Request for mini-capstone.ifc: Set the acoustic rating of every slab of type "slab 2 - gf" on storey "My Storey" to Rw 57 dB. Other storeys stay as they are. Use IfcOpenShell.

First a look at what the model holds.

```python
import ifcopenshell
import ifcopenshell.util.element

model = ifcopenshell.open("mini-capstone.ifc")
print(model.schema)
storey = next(s for s in model.by_type("IfcBuildingStorey") if s.Name == "My Storey")
slabs = [e for e in ifcopenshell.util.element.get_decomposition(storey) if e.is_a("IfcSlab")]
seen = {}
for e in slabs:
    element_type = ifcopenshell.util.element.get_type(e)
    key = (element_type.Name if element_type != e and element_type else None, ifcopenshell.util.element.get_pset(e, "Pset_SlabCommon", "AcousticRating"))
    seen[key] = seen.get(key, 0) + 1
for (name, value), count in sorted(seen.items(), key=str):
    print(count, "x", name, "|", value)
```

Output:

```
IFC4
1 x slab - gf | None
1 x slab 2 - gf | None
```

```python
import ifcopenshell
import ifcopenshell.api.pset
import ifcopenshell.util.element

model = ifcopenshell.open("mini-capstone.ifc")

storey = next(s for s in model.by_type("IfcBuildingStorey") if s.Name == "My Storey")
slabs = [e for e in ifcopenshell.util.element.get_decomposition(storey) if e.is_a("IfcSlab")]

count = 0
for e in slabs:
    element_type = ifcopenshell.util.element.get_type(e)
    if element_type in (None, e) or element_type.Name != "slab 2 - gf":
        continue
    # add_pset returns the element's existing set when there is one.
    pset = ifcopenshell.api.pset.add_pset(model, product=e, name="Pset_SlabCommon")
    ifcopenshell.api.pset.edit_pset(model, pset=pset, properties={"AcousticRating": "Rw 57 dB"})
    count += 1

print(count, "slabs updated")

model.write("mini-capstone_updated.ifc")
```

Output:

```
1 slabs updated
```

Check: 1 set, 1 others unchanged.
